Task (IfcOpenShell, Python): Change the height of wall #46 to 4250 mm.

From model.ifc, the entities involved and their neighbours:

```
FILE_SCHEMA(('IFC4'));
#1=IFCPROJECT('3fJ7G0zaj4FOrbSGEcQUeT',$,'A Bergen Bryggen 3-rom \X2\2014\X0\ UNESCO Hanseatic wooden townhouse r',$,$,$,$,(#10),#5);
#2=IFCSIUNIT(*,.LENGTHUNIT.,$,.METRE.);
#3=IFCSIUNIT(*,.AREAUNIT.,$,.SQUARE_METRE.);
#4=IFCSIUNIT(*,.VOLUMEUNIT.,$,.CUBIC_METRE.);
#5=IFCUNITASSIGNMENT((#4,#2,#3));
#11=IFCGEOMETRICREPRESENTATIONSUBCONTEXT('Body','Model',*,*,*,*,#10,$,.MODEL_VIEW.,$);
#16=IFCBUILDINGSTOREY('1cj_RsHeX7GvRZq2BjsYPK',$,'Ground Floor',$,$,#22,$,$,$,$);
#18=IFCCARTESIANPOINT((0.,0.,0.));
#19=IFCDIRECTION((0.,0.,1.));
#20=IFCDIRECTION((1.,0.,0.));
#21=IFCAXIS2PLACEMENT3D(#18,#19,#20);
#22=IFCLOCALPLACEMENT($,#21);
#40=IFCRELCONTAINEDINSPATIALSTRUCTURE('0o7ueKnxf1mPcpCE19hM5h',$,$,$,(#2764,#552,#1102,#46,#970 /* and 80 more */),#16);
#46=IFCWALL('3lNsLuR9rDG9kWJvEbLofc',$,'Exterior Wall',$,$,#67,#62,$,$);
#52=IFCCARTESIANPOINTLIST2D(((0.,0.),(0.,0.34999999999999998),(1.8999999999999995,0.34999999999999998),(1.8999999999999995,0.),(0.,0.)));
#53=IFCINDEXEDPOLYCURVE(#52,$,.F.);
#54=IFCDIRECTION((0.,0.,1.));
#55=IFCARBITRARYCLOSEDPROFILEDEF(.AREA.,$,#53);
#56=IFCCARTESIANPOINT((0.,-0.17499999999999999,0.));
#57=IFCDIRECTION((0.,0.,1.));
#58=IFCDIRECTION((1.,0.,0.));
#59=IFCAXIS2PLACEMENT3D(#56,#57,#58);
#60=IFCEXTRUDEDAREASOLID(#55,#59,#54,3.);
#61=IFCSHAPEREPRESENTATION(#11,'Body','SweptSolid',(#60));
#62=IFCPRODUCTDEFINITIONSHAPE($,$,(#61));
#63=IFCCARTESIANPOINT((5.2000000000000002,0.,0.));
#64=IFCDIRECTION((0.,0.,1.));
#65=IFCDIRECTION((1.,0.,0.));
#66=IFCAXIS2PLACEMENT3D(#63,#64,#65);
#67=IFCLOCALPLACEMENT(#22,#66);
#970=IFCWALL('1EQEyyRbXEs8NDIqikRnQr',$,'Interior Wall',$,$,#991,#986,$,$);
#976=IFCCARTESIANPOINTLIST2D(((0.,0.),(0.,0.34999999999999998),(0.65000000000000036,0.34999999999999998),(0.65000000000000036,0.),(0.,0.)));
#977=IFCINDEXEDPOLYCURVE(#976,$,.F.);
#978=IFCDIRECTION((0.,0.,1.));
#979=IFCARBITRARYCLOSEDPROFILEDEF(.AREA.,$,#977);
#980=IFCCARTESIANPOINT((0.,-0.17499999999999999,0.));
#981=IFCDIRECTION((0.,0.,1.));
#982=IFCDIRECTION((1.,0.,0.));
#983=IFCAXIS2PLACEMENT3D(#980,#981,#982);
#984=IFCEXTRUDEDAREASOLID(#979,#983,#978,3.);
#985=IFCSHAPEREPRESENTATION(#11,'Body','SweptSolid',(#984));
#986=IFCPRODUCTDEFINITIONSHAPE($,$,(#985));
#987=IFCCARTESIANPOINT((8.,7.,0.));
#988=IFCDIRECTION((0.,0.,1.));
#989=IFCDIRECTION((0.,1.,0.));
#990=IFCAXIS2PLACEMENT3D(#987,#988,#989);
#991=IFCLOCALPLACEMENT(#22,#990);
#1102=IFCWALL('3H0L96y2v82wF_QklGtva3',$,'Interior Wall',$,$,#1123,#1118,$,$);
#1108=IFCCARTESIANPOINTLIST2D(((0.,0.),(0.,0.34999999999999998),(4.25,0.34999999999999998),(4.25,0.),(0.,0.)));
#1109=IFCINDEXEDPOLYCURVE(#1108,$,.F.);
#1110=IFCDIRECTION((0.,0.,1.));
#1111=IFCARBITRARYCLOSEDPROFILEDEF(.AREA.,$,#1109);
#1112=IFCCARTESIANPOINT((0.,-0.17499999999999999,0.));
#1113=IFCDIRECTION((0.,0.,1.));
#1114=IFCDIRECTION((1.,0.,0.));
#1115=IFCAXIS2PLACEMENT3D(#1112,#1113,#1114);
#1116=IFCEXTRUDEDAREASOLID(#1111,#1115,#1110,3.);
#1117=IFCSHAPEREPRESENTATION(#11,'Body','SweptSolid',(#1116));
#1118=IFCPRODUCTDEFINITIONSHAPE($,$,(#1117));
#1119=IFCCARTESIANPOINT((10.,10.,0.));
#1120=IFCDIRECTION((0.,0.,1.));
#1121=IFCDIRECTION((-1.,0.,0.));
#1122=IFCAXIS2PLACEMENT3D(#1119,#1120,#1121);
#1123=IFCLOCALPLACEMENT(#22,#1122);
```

```python
import ifcopenshell
import ifcopenshell.geom
import ifcopenshell.util.representation
import ifcopenshell.util.shape

model = ifcopenshell.open("model.ifc")
settings = ifcopenshell.geom.settings()


def volume(element):
    """Net volume in cubic metres, openings subtracted."""
    shape = ifcopenshell.geom.create_shape(settings, element)
    return ifcopenshell.util.shape.get_volume(shape.geometry)


wall = model.by_guid("3lNsLuR9rDG9kWJvEbLofc")
before = volume(wall)

body = ifcopenshell.util.representation.get_representation(wall, "Model", "Body")
solid = body.Items[0]
old_height = solid.Depth
solid.Depth = 4.25
after = volume(wall)

print(f"height {old_height:g} -> {solid.Depth:g}, volume {before:.3f} -> {after:.3f} m3")

model.write("model_rev.ifc")
```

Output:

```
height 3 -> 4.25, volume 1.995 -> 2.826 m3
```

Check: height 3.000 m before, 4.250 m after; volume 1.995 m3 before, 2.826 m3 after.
